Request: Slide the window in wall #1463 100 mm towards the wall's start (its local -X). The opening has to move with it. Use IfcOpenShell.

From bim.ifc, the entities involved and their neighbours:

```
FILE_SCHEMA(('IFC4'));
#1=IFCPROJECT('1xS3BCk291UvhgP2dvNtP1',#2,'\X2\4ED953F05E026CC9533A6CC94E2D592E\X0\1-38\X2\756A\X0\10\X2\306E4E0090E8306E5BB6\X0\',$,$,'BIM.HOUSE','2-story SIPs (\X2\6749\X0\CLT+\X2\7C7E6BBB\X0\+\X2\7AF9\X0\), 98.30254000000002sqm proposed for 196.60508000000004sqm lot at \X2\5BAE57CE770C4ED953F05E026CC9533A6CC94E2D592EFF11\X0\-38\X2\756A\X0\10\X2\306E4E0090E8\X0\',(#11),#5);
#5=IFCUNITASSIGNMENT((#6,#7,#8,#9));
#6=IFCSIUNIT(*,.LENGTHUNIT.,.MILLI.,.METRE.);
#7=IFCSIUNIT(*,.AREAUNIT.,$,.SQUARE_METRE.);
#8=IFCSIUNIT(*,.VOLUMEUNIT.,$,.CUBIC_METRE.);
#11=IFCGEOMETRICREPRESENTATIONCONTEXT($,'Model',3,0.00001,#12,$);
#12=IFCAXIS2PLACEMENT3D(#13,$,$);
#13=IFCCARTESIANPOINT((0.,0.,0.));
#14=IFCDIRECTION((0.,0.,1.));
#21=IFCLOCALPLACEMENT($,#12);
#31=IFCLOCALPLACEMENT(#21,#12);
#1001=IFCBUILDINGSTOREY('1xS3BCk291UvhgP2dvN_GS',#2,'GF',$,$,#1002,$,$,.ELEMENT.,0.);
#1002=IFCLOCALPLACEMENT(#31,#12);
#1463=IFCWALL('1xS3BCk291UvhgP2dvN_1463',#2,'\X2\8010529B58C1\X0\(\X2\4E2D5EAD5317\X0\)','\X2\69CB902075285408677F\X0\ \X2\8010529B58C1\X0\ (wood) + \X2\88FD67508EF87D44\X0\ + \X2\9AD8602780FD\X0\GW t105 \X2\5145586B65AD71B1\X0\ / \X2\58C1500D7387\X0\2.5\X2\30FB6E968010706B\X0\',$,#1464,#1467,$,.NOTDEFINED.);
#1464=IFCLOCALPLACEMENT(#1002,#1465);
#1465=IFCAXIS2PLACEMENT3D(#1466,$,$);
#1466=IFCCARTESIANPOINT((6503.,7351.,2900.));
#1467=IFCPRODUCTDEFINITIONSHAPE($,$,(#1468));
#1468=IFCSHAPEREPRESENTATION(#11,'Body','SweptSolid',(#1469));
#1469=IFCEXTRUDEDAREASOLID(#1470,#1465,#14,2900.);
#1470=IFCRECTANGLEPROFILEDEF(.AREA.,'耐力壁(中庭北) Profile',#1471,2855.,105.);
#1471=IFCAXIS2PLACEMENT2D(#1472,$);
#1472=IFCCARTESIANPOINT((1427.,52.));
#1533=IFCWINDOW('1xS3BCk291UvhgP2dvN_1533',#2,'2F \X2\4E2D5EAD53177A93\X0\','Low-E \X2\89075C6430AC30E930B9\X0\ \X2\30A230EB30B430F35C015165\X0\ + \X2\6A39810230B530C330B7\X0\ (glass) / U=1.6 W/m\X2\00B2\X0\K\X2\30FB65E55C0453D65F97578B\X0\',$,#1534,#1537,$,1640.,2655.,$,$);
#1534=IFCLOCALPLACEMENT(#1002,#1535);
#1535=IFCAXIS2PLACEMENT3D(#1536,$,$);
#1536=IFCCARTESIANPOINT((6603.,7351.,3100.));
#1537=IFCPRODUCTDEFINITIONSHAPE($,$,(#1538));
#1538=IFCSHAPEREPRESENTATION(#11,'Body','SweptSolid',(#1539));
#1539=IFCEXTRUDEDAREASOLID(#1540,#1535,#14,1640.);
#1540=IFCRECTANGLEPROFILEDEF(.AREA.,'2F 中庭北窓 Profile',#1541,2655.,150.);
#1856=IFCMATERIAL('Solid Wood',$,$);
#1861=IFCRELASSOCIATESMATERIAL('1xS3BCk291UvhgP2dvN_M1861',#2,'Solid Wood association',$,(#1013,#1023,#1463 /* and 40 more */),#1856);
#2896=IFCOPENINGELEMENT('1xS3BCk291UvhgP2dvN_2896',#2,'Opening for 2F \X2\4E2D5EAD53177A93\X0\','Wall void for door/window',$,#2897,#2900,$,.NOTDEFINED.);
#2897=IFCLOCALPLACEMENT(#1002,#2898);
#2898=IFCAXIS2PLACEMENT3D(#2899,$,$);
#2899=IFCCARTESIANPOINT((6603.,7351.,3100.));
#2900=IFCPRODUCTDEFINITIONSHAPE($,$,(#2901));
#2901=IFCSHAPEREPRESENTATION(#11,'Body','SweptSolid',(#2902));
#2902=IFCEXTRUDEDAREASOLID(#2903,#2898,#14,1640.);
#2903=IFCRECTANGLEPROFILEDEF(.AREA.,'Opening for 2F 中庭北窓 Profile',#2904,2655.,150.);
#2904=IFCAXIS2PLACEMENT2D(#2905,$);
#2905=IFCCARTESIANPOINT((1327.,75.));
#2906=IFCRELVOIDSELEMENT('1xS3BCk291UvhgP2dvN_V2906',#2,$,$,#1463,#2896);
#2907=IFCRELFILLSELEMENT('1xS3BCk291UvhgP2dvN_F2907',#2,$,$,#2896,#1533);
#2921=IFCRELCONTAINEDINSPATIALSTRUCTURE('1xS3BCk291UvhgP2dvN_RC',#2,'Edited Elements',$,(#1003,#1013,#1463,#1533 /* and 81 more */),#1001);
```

```python
import ifcopenshell
import ifcopenshell.api.geometry
import ifcopenshell.util.placement

model = ifcopenshell.open("bim.ifc")

window = model.by_guid("1xS3BCk291UvhgP2dvN_1533")
opening = window.FillsVoids[0].RelatingOpeningElement
wall = opening.VoidsElements[0].RelatingBuildingElement

wall_matrix = ifcopenshell.util.placement.get_local_placement(wall.ObjectPlacement)
shift = wall_matrix[:3, 0] * -100.0
before = ifcopenshell.util.placement.get_local_placement(window.ObjectPlacement)[:3, 3].copy()

# The window is not placed relative to its opening, so move both.
for product in (opening, window):
    matrix = ifcopenshell.util.placement.get_local_placement(product.ObjectPlacement)
    matrix[:3, 3] += shift
    ifcopenshell.api.geometry.edit_object_placement(model, product=product, matrix=matrix, is_si=False)

after = ifcopenshell.util.placement.get_local_placement(window.ObjectPlacement)[:3, 3]
print("window moved by", (after - before).round(3) + 0.0)

model.write("bim_edited.ifc")
```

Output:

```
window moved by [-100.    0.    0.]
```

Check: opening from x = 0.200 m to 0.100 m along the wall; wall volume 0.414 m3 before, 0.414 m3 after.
